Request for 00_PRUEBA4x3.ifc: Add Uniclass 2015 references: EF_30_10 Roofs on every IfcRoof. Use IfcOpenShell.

First a look at what the model holds.

```python
import ifcopenshell

model = ifcopenshell.open("00_PRUEBA4x3.ifc")
print(model.schema)
print("classifications:", [c.Name for c in model.by_type("IfcClassification")])
for ifc_class in ("IfcDoor", "IfcRoof", "IfcStair", "IfcWall", "IfcWindow"):
    print(ifc_class, len(model.by_type(ifc_class)))
```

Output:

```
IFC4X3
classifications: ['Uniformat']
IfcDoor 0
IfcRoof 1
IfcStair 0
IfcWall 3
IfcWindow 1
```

```python
import ifcopenshell
import ifcopenshell.api.classification

model = ifcopenshell.open("00_PRUEBA4x3.ifc")

system = ifcopenshell.api.classification.add_classification(model, classification="Uniclass 2015")

codes = {
    "IfcRoof": ("EF_30_10", "Roofs"),
}
for ifc_class, (code, name) in codes.items():
    products = model.by_type(ifc_class)
    ifcopenshell.api.classification.add_reference(
        model, products=products, classification=system, identification=code, name=name
    )
    print(code, len(products))

model.write("00_PRUEBA4x3_v2.ifc")
```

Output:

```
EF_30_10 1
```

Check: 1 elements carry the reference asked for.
